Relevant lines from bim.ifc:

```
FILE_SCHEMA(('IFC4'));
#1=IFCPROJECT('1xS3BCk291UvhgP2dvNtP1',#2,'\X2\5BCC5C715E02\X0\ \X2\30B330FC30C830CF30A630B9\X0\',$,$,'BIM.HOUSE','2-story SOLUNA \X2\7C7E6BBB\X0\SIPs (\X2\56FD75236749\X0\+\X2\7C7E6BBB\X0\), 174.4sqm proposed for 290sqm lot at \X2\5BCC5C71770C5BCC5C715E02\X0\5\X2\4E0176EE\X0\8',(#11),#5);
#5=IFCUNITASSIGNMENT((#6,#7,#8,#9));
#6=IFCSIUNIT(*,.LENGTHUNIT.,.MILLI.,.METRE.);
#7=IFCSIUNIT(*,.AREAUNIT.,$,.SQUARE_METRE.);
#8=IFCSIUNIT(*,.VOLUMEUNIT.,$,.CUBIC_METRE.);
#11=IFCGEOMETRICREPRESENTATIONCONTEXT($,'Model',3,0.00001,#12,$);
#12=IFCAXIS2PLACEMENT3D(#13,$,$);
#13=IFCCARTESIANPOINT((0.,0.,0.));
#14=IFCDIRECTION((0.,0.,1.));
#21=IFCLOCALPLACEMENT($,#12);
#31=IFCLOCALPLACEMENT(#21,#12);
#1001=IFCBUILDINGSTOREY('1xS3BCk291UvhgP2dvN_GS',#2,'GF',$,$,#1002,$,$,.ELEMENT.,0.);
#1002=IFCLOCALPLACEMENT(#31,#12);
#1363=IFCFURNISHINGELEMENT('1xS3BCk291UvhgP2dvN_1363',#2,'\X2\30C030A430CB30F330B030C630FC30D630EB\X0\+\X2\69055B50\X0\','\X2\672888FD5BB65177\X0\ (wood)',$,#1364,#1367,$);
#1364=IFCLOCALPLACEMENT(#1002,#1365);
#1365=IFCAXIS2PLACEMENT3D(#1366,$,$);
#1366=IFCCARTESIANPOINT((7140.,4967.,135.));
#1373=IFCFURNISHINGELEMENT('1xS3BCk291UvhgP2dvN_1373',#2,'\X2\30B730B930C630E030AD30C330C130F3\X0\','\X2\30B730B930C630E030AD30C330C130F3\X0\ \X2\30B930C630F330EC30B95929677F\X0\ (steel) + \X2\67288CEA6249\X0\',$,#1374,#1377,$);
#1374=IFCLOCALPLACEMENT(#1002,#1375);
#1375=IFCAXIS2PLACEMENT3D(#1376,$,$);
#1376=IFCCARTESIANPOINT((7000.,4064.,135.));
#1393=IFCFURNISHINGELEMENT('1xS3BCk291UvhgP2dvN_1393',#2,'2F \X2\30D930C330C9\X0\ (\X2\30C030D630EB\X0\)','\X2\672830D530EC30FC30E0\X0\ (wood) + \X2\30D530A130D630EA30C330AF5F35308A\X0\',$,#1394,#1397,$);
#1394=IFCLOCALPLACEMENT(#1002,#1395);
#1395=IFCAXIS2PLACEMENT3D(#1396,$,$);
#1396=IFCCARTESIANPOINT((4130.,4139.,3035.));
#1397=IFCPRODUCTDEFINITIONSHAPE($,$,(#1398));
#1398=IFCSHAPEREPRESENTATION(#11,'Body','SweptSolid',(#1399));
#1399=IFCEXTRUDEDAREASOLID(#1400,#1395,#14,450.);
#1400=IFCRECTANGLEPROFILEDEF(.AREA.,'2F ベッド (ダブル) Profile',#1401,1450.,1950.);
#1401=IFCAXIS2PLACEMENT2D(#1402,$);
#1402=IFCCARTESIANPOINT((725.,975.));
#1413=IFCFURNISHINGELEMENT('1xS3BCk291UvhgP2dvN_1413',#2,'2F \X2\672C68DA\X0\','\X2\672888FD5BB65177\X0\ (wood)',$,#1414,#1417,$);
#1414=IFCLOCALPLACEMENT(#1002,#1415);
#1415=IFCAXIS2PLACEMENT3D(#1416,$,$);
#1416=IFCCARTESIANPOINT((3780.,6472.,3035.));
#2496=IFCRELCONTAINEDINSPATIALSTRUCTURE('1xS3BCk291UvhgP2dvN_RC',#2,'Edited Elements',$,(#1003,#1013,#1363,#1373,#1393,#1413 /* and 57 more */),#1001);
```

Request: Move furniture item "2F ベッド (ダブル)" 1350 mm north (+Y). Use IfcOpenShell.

```python
import ifcopenshell
import ifcopenshell.api.geometry
import ifcopenshell.util.placement
import ifcopenshell.util.unit

model = ifcopenshell.open("bim.ifc")
unit_scale = ifcopenshell.util.unit.calculate_unit_scale(model)

item = model.by_guid("1xS3BCk291UvhgP2dvN_1393")
matrix = ifcopenshell.util.placement.get_local_placement(item.ObjectPlacement)
matrix[1, 3] += 1.35 / unit_scale
ifcopenshell.api.geometry.edit_object_placement(model, product=item, matrix=matrix, is_si=False)

print(ifcopenshell.util.placement.get_local_placement(item.ObjectPlacement).round(3) + 0.0)

model.write("bim_v2.ifc")
```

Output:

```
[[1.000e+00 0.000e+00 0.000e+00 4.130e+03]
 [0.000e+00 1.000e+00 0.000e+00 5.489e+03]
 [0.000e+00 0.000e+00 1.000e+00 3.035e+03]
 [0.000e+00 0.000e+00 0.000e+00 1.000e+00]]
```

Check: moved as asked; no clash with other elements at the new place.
